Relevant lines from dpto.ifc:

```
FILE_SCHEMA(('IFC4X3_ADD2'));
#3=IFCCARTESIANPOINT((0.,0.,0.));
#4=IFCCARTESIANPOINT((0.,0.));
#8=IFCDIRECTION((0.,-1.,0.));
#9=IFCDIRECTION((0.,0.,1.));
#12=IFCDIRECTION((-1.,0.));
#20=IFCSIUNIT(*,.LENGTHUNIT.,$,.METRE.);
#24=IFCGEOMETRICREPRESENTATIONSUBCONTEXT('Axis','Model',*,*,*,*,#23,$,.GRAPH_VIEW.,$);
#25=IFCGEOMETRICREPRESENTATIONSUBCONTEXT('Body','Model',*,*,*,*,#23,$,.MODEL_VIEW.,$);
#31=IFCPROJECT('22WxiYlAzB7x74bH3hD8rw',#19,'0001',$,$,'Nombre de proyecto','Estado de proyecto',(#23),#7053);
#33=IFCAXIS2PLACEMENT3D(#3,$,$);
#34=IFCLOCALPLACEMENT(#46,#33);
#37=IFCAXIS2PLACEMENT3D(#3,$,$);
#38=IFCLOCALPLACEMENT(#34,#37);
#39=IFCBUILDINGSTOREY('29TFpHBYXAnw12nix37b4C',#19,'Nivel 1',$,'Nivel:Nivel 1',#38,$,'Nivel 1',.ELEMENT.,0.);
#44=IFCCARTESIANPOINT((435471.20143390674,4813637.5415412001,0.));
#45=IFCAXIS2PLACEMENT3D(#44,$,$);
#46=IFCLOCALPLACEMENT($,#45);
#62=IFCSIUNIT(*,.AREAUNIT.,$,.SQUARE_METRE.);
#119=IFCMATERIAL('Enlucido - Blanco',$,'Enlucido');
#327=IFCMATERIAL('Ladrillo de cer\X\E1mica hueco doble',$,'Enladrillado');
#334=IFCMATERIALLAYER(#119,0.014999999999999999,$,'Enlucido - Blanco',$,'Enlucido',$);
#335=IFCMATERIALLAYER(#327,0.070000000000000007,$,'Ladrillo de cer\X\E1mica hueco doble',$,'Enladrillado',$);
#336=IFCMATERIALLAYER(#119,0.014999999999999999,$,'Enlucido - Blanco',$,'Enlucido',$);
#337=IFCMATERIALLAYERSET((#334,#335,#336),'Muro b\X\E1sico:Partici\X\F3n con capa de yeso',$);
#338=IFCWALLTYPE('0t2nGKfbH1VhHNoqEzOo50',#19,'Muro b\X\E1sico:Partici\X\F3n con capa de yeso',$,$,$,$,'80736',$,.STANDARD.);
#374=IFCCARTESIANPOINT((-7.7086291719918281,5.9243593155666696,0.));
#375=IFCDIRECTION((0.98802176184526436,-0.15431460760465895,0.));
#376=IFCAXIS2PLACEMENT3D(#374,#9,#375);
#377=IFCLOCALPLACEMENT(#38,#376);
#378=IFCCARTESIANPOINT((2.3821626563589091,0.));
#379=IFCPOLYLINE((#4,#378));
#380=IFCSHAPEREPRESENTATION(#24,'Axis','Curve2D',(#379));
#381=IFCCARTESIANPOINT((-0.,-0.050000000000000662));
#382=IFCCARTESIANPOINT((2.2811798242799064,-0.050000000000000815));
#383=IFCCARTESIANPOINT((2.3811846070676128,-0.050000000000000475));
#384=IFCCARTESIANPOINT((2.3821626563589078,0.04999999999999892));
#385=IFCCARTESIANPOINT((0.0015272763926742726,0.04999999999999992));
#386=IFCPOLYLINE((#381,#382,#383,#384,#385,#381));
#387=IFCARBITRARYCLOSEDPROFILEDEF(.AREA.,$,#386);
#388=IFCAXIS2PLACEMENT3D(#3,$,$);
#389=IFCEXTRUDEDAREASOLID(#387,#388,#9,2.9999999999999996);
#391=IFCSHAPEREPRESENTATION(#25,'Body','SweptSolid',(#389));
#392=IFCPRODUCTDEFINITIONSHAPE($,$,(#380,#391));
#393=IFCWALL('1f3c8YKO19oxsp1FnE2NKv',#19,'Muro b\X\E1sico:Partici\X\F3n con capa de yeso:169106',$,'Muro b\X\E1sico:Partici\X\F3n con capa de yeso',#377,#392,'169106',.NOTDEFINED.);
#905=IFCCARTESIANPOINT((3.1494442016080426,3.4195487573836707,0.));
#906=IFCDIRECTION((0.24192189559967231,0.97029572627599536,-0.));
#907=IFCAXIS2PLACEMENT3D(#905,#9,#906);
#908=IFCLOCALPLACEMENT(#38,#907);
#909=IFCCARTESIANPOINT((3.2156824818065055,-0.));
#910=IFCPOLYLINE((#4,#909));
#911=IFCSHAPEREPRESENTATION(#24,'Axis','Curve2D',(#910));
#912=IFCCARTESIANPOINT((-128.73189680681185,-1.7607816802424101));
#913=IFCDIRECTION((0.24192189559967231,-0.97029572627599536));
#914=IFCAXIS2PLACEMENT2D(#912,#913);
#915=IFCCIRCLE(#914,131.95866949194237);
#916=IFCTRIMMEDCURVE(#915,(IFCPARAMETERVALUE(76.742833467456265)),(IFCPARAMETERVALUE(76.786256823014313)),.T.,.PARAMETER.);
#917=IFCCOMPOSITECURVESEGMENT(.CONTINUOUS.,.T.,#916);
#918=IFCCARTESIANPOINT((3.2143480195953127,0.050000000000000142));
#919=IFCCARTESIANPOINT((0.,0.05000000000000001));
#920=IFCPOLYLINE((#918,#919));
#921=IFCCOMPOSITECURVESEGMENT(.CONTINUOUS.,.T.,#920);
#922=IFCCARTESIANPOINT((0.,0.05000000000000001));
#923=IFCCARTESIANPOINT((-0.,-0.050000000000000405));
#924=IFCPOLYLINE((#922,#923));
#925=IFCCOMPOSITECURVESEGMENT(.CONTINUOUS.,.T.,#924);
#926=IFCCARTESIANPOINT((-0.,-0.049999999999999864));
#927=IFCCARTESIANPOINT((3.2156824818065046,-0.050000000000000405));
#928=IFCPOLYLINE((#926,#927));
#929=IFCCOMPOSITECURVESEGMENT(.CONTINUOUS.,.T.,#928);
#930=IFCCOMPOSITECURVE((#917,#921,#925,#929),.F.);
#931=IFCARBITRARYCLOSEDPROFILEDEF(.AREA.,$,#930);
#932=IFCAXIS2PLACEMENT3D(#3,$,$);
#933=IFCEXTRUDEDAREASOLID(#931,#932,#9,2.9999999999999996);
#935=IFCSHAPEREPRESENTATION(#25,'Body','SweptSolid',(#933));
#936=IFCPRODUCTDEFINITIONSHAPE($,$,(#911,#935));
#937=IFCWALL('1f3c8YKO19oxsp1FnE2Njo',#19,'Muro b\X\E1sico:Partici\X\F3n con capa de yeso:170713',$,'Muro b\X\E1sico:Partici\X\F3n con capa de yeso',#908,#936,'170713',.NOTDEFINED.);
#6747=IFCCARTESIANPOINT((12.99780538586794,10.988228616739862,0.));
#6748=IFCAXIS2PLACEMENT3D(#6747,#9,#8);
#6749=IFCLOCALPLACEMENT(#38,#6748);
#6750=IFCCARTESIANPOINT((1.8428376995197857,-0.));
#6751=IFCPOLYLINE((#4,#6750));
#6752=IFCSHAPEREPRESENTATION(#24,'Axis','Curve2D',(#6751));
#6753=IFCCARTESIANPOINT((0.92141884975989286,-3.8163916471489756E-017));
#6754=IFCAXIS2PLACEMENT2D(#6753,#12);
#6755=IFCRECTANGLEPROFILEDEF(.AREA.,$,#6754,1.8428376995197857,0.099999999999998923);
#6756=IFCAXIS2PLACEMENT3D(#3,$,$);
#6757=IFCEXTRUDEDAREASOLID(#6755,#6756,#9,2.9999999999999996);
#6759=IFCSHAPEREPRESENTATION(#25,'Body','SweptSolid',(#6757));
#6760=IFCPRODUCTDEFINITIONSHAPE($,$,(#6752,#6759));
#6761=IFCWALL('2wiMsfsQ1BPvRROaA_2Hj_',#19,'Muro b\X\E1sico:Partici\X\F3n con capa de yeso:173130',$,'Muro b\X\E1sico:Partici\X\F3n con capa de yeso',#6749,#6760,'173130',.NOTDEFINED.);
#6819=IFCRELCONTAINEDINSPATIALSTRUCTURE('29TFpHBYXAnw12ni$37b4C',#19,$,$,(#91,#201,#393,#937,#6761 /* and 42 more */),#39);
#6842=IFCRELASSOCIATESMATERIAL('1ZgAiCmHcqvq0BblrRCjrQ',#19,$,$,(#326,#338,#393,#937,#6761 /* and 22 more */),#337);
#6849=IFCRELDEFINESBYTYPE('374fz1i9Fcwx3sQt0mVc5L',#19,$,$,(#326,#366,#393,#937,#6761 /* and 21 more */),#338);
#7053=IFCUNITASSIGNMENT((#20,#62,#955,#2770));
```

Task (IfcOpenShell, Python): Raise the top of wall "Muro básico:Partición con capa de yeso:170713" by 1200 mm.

```python
import ifcopenshell
import ifcopenshell.geom
import ifcopenshell.util.representation
import ifcopenshell.util.shape
import ifcopenshell.util.unit

model = ifcopenshell.open("dpto.ifc")
unit_scale = ifcopenshell.util.unit.calculate_unit_scale(model)
settings = ifcopenshell.geom.settings()


def volume(element):
    """Net volume in cubic metres, openings subtracted."""
    shape = ifcopenshell.geom.create_shape(settings, element)
    return ifcopenshell.util.shape.get_volume(shape.geometry)


wall = model.by_id(937)
before = volume(wall)

body = ifcopenshell.util.representation.get_representation(wall, "Model", "Body")
solid = body.Items[0]
old_height = solid.Depth
solid.Depth += 1.2 / unit_scale
after = volume(wall)

print(f"height {old_height:g} -> {solid.Depth:g}, volume {before:.3f} -> {after:.3f} m3")

model.write("dpto-out.ifc")
```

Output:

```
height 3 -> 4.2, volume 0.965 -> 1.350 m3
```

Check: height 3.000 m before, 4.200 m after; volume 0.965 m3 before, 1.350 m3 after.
